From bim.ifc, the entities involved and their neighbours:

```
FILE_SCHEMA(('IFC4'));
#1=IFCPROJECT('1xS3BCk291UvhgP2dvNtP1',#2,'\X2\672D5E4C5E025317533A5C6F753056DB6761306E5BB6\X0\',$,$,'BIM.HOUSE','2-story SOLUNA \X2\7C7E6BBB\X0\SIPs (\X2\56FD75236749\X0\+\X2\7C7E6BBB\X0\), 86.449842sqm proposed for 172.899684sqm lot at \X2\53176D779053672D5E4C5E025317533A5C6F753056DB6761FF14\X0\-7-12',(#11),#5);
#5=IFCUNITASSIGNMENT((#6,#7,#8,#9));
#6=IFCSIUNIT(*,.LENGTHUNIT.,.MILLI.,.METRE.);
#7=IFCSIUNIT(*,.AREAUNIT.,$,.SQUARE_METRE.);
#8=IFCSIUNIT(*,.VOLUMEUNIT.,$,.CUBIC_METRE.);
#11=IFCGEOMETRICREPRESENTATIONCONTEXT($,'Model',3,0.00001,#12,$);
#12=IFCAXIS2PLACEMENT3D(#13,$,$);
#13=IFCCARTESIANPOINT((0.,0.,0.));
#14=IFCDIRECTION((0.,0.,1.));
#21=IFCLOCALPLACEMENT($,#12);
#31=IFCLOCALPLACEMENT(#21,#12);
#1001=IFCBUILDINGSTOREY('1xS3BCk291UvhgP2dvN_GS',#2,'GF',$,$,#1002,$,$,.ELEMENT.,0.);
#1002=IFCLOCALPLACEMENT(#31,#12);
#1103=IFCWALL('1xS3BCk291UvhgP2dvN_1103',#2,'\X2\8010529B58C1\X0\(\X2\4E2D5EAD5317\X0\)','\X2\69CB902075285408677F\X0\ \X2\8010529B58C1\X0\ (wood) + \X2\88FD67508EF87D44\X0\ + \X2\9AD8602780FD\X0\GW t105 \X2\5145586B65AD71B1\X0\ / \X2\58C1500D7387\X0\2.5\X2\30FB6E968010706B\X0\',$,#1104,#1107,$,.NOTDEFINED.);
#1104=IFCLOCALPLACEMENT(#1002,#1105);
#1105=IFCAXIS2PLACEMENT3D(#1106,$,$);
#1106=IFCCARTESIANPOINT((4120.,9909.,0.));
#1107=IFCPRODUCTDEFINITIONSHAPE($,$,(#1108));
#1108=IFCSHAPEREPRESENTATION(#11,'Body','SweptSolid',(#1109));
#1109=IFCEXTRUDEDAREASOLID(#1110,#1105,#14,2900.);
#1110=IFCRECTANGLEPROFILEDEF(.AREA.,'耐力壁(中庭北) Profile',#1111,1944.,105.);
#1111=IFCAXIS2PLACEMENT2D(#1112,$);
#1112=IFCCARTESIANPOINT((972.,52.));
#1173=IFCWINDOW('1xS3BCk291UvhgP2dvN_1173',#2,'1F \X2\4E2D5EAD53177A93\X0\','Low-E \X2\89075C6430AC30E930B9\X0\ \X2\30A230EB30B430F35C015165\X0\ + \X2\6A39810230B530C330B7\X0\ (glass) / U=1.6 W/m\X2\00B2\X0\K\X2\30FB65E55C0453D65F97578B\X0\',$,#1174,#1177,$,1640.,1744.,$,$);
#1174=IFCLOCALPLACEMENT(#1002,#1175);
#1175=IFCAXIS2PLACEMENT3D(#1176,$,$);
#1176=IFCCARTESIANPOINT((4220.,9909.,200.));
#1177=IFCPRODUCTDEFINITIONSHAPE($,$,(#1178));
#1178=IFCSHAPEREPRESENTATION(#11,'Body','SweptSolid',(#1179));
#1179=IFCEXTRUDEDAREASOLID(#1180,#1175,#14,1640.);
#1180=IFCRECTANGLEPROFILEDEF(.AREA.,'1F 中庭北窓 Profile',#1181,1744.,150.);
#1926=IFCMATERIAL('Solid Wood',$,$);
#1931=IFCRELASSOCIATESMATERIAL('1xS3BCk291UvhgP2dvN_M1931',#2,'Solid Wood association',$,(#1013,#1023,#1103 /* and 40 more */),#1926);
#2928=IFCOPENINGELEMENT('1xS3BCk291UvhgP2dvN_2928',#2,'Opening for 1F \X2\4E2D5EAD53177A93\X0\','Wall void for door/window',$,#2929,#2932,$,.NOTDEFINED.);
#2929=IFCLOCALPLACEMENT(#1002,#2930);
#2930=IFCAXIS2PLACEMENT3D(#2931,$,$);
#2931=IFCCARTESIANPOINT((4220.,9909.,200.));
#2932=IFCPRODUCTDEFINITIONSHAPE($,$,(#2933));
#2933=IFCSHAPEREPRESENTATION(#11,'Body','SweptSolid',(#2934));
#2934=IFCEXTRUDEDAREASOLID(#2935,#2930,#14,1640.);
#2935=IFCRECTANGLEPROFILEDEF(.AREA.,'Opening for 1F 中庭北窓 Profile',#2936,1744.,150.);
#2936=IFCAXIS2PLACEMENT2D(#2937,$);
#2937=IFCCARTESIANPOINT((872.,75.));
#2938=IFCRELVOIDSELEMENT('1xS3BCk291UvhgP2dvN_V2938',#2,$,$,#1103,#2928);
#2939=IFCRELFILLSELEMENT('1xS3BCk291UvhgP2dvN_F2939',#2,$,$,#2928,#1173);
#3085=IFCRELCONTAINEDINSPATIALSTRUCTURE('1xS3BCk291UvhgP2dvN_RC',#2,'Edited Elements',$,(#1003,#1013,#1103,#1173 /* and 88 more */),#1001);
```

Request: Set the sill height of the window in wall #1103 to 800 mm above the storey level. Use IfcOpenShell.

```python
import numpy as np
import ifcopenshell
import ifcopenshell.api.geometry
import ifcopenshell.geom
import ifcopenshell.util.element
import ifcopenshell.util.placement
import ifcopenshell.util.shape
import ifcopenshell.util.unit

model = ifcopenshell.open("bim.ifc")
unit_scale = ifcopenshell.util.unit.calculate_unit_scale(model)

window = model.by_id(1173)
opening = window.FillsVoids[0].RelatingOpeningElement
storey = ifcopenshell.util.element.get_container(window, ifc_class="IfcBuildingStorey")
level = ifcopenshell.util.placement.get_local_placement(storey.ObjectPlacement)[2, 3]

# The opening's origin need not be at the sill, so measure its lowest point.
shape = ifcopenshell.geom.create_shape(ifcopenshell.geom.settings(), opening)
bottom = ifcopenshell.util.shape.get_shape_bottom_elevation(shape, shape.geometry) / unit_scale
dz = level + 0.8 / unit_scale - bottom

shift = np.array([0.0, 0.0, dz])
# The window is not placed relative to its opening, so move both.
for product in (opening, window):
    matrix = ifcopenshell.util.placement.get_local_placement(product.ObjectPlacement)
    matrix[:3, 3] += shift
    ifcopenshell.api.geometry.edit_object_placement(model, product=product, matrix=matrix, is_si=False)

print(f"moved by {dz * unit_scale:+.3f} m")

model.write("bim_updated.ifc")
```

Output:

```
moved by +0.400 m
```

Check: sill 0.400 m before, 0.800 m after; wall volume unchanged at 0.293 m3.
